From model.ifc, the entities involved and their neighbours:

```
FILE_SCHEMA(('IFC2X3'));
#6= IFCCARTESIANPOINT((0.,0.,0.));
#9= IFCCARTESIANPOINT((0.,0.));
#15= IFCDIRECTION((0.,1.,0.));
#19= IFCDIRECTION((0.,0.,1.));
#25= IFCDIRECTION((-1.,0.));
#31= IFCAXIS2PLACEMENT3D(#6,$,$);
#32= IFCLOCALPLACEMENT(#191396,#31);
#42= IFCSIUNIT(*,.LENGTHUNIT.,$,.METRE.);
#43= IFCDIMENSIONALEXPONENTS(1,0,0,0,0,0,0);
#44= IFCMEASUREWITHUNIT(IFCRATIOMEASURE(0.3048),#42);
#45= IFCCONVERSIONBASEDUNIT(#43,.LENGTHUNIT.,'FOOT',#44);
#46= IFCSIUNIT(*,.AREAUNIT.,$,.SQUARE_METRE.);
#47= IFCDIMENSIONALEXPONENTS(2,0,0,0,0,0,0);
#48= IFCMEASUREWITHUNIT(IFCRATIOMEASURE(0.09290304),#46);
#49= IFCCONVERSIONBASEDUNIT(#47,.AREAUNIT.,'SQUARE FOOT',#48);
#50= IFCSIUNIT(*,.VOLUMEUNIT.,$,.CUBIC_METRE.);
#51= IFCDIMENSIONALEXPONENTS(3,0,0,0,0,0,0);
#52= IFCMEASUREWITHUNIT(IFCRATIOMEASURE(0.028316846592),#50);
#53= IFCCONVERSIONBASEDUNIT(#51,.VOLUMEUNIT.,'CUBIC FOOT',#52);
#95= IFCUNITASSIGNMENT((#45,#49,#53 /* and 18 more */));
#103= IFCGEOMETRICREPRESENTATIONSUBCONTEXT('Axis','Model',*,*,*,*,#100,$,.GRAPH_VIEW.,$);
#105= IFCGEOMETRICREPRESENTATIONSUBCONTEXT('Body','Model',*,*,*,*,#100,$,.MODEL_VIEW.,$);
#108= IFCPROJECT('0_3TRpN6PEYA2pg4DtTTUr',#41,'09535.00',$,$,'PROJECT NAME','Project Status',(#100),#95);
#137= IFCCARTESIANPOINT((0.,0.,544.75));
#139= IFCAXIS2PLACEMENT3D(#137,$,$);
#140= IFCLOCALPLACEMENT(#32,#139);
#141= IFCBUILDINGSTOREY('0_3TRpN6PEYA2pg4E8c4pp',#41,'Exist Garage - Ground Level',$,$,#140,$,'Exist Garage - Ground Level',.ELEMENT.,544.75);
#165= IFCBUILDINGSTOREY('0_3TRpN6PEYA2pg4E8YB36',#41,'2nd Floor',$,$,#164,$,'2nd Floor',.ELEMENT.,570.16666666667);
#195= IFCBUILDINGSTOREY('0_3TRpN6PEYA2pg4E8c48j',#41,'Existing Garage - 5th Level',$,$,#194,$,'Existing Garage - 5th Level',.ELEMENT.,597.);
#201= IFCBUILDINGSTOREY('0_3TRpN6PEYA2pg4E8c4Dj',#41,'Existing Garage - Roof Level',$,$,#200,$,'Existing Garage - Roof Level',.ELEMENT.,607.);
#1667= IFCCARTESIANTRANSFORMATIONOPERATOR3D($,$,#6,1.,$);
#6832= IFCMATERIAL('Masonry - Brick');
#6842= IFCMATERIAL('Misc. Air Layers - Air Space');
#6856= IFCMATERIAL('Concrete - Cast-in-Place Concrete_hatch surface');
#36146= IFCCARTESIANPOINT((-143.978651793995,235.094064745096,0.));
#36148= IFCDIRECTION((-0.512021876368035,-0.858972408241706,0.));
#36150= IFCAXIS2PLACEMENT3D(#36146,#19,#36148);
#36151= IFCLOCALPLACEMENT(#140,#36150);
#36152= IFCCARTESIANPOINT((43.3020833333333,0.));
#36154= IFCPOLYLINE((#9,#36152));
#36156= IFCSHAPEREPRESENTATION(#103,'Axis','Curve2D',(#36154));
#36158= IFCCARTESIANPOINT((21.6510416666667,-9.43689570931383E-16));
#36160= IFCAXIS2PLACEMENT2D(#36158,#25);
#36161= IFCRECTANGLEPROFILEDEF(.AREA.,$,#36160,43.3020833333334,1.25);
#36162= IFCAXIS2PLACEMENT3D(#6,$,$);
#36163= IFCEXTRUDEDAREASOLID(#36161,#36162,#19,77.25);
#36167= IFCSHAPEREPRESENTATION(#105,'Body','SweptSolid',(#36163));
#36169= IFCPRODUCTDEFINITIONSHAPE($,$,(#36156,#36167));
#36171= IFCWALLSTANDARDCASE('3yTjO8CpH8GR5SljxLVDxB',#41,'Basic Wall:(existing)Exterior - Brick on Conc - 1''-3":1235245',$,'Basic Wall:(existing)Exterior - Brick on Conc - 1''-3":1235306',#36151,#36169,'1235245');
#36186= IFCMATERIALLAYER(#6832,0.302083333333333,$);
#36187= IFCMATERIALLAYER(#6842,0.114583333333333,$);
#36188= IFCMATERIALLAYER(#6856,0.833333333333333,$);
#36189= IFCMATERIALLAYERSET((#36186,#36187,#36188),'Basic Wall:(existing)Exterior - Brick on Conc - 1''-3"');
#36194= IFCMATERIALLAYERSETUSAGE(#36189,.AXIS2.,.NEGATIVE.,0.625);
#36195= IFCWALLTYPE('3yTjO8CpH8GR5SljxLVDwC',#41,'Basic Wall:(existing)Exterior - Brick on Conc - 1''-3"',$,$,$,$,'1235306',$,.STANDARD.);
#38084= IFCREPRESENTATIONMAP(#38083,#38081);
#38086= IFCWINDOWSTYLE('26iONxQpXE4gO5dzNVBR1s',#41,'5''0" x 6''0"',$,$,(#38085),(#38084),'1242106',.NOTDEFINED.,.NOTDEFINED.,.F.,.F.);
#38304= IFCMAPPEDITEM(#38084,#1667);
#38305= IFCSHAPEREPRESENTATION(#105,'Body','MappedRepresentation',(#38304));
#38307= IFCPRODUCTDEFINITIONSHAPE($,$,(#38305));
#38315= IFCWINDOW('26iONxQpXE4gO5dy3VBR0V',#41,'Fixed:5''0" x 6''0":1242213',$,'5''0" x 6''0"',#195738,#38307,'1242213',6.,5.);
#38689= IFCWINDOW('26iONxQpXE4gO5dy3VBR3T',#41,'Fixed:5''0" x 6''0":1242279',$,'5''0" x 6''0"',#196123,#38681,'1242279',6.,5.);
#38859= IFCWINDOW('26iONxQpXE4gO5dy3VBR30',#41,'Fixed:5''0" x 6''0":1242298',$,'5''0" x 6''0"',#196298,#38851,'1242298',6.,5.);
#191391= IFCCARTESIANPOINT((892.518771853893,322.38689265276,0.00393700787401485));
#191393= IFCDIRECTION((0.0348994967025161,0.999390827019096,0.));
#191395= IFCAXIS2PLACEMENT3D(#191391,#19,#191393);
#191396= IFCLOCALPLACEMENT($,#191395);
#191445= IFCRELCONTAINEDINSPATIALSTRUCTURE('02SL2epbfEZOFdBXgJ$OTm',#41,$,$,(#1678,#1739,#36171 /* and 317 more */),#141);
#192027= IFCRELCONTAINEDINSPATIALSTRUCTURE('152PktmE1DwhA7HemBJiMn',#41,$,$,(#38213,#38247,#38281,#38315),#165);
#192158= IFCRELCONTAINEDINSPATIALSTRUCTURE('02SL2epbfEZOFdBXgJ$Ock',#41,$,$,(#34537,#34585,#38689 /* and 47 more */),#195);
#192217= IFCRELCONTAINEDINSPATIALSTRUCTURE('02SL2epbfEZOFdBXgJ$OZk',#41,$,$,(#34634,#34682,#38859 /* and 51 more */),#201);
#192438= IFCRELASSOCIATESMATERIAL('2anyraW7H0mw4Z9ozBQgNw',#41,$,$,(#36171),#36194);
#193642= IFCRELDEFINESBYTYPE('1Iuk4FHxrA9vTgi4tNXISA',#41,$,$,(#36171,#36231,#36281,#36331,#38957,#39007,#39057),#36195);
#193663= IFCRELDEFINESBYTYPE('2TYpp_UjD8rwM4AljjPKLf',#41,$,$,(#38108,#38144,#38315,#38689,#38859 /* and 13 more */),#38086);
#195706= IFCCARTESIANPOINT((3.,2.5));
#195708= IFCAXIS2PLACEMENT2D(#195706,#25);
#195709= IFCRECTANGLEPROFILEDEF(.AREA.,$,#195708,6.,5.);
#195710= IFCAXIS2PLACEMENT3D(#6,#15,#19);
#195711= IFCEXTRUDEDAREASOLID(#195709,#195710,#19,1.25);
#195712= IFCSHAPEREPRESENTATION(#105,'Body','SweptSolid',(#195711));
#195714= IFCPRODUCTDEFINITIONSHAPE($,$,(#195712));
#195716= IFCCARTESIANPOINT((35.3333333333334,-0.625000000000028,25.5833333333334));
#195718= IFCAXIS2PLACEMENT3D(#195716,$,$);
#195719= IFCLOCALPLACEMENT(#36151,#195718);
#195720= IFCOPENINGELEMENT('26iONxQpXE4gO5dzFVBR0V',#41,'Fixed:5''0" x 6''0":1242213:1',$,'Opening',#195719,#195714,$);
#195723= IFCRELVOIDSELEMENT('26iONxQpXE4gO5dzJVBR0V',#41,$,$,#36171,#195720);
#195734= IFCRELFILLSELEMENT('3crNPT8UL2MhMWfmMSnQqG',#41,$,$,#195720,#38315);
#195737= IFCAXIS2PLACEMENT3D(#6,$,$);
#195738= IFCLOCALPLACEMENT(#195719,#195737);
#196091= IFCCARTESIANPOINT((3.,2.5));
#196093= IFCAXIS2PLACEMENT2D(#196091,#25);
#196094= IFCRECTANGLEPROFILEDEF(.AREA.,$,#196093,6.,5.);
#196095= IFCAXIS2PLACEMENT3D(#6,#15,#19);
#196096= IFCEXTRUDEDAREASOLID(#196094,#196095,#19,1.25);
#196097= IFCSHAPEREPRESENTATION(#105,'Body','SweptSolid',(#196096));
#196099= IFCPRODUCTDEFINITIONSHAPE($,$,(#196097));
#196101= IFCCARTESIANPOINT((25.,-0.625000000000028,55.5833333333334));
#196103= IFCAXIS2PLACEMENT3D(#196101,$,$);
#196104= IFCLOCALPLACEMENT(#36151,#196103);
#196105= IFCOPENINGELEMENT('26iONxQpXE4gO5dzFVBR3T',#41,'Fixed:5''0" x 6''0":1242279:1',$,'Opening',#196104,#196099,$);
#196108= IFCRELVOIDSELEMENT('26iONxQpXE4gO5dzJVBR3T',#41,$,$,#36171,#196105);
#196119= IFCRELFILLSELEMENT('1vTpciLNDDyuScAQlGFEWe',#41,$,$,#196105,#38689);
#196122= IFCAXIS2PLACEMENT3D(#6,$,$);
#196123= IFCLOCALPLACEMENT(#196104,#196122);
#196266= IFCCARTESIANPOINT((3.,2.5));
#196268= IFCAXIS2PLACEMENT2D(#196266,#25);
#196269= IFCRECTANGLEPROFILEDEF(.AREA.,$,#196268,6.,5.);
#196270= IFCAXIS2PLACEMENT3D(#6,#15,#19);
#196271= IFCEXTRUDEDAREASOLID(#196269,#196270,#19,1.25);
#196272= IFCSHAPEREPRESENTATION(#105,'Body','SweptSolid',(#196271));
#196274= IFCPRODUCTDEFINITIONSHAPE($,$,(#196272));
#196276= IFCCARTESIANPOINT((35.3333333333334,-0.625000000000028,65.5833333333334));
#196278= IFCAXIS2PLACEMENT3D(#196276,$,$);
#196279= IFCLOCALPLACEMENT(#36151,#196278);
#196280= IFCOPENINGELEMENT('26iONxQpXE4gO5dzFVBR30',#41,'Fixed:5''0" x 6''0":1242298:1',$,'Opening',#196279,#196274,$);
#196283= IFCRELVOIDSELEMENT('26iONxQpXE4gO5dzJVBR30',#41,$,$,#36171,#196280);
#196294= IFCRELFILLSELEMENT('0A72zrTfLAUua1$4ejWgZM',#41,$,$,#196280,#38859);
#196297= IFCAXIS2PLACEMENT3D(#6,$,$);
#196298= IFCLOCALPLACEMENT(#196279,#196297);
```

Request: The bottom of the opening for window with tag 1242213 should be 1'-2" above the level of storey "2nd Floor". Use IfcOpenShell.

```python
import numpy as np
import ifcopenshell
import ifcopenshell.api.geometry
import ifcopenshell.geom
import ifcopenshell.util.element
import ifcopenshell.util.placement
import ifcopenshell.util.shape
import ifcopenshell.util.unit

model = ifcopenshell.open("model.ifc")
unit_scale = ifcopenshell.util.unit.calculate_unit_scale(model)

window = model.by_id(38315)
opening = window.FillsVoids[0].RelatingOpeningElement
storey = ifcopenshell.util.element.get_container(window, ifc_class="IfcBuildingStorey")
level = ifcopenshell.util.placement.get_local_placement(storey.ObjectPlacement)[2, 3]

# The opening's origin need not be at the sill, so measure its lowest point.
shape = ifcopenshell.geom.create_shape(ifcopenshell.geom.settings(), opening)
bottom = ifcopenshell.util.shape.get_shape_bottom_elevation(shape, shape.geometry) / unit_scale
dz = level + 14 * 0.0254 / unit_scale - bottom

shift = np.array([0.0, 0.0, dz])
# The window is placed relative to its opening, so it follows when the opening moves.
matrix = ifcopenshell.util.placement.get_local_placement(opening.ObjectPlacement)
matrix[:3, 3] += shift
ifcopenshell.api.geometry.edit_object_placement(
    model, product=opening, matrix=matrix, is_si=False, should_transform_children=True
)

print(f"moved by {dz * unit_scale:+.3f} m")

model.write("model_rev.ifc")
```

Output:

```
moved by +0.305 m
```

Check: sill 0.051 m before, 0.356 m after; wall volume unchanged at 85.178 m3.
